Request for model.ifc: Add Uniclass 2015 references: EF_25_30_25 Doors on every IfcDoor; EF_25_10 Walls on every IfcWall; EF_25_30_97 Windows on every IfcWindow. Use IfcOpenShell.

First a look at what the model holds.

```python
import ifcopenshell

model = ifcopenshell.open("model.ifc")
print(model.schema)
print("classifications:", [c.Name for c in model.by_type("IfcClassification")])
for ifc_class in ("IfcDoor", "IfcRoof", "IfcStair", "IfcWall", "IfcWindow"):
    print(ifc_class, len(model.by_type(ifc_class)))
```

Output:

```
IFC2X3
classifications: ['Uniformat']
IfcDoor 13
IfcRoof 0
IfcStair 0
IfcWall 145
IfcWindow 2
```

```python
import ifcopenshell
import ifcopenshell.api.classification

model = ifcopenshell.open("model.ifc")

# IFC2X3 requires Source and Edition and has no link from the project to the system.
system = model.create_entity("IfcClassification", Source="NBS", Edition="2015", Name="Uniclass 2015")

codes = {
    "IfcDoor": ("EF_25_30_25", "Doors"),
    "IfcWall": ("EF_25_10", "Walls"),
    "IfcWindow": ("EF_25_30_97", "Windows"),
}
for ifc_class, (code, name) in codes.items():
    products = model.by_type(ifc_class)
    ifcopenshell.api.classification.add_reference(
        model, products=products, classification=system, identification=code, name=name
    )
    print(code, len(products))

model.write("model-out.ifc")
```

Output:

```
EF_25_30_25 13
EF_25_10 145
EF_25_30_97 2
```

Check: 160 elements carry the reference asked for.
